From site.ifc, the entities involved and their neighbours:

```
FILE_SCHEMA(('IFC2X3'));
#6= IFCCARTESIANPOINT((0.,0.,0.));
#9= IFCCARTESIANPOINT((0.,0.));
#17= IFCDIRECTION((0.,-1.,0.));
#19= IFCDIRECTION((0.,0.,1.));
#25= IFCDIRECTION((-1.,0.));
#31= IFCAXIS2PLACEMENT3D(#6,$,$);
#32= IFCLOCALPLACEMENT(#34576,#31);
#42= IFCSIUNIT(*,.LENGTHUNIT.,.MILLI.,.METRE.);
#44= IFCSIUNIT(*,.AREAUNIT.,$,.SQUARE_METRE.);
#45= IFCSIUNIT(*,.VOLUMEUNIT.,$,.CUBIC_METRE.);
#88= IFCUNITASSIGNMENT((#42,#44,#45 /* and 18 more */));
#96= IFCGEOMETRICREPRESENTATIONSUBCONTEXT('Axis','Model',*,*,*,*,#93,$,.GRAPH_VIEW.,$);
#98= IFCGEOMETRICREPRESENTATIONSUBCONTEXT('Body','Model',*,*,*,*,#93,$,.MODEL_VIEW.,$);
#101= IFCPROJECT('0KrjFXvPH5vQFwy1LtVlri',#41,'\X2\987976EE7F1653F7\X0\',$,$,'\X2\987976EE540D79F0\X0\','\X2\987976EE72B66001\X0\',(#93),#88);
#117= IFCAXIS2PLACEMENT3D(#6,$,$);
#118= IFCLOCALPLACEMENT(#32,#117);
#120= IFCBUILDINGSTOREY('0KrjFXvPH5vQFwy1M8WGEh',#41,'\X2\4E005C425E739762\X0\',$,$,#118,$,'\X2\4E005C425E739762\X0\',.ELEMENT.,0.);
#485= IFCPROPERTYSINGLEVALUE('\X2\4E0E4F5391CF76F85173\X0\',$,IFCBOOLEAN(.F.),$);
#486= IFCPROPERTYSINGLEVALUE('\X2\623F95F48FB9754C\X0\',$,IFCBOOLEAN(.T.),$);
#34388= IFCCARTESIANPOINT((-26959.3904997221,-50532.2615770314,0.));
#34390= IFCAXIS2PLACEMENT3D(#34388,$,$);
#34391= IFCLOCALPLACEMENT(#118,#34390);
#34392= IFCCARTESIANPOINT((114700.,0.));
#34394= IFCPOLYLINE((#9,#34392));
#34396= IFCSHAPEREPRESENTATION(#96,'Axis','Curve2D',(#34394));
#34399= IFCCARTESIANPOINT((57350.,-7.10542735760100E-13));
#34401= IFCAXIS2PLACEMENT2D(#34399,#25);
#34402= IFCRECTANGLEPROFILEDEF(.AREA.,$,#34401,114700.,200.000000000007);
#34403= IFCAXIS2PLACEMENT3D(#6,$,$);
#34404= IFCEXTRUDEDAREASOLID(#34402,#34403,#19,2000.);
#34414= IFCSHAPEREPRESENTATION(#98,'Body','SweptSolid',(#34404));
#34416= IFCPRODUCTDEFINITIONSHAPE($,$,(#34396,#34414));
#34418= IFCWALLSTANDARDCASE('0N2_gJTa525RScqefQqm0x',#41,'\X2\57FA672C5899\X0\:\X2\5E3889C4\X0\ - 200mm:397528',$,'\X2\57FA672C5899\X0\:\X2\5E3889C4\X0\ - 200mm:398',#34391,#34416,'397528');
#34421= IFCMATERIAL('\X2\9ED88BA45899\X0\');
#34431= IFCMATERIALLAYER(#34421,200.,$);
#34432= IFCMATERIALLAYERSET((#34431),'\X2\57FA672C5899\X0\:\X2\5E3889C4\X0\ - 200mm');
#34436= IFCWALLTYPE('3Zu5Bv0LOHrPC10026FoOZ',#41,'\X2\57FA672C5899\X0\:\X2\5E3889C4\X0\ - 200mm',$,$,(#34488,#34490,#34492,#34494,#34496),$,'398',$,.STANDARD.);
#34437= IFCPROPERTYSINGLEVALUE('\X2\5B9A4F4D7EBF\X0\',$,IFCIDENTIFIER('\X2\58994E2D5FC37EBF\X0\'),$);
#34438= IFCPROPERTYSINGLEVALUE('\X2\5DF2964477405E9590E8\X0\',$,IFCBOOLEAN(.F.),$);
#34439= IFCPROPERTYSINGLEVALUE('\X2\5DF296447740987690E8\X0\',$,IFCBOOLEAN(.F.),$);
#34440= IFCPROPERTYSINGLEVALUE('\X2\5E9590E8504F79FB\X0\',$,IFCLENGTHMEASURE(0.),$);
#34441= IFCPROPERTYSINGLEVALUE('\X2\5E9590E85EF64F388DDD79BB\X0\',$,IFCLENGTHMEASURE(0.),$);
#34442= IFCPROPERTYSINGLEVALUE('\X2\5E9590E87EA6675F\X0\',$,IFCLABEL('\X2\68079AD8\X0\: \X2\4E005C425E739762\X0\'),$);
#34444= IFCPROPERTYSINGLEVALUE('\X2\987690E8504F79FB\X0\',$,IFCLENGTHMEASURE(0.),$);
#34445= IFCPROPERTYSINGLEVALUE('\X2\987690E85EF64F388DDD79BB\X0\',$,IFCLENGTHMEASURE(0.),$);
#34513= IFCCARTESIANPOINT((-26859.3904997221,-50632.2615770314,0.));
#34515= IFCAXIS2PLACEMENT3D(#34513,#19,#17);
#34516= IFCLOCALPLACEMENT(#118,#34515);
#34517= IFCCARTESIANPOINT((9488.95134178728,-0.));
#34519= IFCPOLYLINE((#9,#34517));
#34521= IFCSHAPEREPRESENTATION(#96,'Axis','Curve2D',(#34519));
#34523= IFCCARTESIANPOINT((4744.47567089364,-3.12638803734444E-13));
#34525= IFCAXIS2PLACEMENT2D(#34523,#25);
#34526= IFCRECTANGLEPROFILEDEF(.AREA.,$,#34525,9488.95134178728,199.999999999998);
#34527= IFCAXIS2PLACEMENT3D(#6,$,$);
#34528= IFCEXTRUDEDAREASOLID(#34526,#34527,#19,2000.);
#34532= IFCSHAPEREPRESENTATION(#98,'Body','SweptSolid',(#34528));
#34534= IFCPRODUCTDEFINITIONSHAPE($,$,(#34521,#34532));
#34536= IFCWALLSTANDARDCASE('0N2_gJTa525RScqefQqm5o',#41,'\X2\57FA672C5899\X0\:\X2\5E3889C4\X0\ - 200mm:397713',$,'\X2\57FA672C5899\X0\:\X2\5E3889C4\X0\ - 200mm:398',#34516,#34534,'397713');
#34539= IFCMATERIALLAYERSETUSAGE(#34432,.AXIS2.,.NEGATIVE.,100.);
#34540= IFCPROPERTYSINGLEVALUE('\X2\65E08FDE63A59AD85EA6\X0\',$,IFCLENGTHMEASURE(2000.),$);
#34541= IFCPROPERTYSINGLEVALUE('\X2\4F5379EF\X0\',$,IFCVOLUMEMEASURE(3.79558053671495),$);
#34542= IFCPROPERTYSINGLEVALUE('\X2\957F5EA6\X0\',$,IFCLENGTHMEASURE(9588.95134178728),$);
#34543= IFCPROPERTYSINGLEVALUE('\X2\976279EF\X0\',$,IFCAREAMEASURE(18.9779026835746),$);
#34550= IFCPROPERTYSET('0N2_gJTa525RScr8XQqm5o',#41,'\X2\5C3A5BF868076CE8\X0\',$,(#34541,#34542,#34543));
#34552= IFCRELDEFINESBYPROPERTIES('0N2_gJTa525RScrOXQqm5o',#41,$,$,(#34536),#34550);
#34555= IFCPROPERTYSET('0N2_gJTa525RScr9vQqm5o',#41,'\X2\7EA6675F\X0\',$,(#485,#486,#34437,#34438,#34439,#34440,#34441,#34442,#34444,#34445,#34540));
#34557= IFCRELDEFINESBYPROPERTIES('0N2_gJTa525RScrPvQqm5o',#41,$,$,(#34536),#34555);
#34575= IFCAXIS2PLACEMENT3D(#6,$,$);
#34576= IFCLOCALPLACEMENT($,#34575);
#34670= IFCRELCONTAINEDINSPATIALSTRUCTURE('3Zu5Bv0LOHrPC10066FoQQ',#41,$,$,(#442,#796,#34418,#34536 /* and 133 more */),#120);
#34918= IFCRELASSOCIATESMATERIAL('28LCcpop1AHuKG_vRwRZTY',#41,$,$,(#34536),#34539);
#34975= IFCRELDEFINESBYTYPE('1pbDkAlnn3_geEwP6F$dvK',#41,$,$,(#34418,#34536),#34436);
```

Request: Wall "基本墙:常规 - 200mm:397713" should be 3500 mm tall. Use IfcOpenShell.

```python
import ifcopenshell
import ifcopenshell.api.pset
import ifcopenshell.geom
import ifcopenshell.util.element
import ifcopenshell.util.representation
import ifcopenshell.util.shape
import ifcopenshell.util.unit

model = ifcopenshell.open("site.ifc")
unit_scale = ifcopenshell.util.unit.calculate_unit_scale(model)
area_scale = ifcopenshell.util.unit.calculate_unit_scale(model, "AREAUNIT")
volume_scale = ifcopenshell.util.unit.calculate_unit_scale(model, "VOLUMEUNIT")
settings = ifcopenshell.geom.settings()


def volume(element):
    """Net volume in cubic metres, openings subtracted."""
    shape = ifcopenshell.geom.create_shape(settings, element)
    return ifcopenshell.util.shape.get_volume(shape.geometry)


wall = model.by_id(34536)
before = volume(wall)

body = ifcopenshell.util.representation.get_representation(wall, "Model", "Body")
solid = body.Items[0]
old_height = solid.Depth
solid.Depth = 3.5 / unit_scale
after = volume(wall)
thickness = 0.2  # wall thickness in metres

# Update the stored height, areas and volumes.
pset = model.by_id(ifcopenshell.util.element.get_pset(wall, "尺寸标注", should_inherit=False)["id"])
ifcopenshell.api.pset.edit_pset(model, pset=pset, properties={
    "体积": model.create_entity("IfcVolumeMeasure", after / volume_scale),
    "面积": model.create_entity("IfcAreaMeasure", after / thickness / area_scale),
})
pset = model.by_id(ifcopenshell.util.element.get_pset(wall, "约束", should_inherit=False)["id"])
ifcopenshell.api.pset.edit_pset(model, pset=pset, properties={
    "无连接高度": model.create_entity("IfcLengthMeasure", solid.Depth),
})

print(f"height {old_height:g} -> {solid.Depth:g}, volume {before:.3f} -> {after:.3f} m3")

model.write("site_updated.ifc")
```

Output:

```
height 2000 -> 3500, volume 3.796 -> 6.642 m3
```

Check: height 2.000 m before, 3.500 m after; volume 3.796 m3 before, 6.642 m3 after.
